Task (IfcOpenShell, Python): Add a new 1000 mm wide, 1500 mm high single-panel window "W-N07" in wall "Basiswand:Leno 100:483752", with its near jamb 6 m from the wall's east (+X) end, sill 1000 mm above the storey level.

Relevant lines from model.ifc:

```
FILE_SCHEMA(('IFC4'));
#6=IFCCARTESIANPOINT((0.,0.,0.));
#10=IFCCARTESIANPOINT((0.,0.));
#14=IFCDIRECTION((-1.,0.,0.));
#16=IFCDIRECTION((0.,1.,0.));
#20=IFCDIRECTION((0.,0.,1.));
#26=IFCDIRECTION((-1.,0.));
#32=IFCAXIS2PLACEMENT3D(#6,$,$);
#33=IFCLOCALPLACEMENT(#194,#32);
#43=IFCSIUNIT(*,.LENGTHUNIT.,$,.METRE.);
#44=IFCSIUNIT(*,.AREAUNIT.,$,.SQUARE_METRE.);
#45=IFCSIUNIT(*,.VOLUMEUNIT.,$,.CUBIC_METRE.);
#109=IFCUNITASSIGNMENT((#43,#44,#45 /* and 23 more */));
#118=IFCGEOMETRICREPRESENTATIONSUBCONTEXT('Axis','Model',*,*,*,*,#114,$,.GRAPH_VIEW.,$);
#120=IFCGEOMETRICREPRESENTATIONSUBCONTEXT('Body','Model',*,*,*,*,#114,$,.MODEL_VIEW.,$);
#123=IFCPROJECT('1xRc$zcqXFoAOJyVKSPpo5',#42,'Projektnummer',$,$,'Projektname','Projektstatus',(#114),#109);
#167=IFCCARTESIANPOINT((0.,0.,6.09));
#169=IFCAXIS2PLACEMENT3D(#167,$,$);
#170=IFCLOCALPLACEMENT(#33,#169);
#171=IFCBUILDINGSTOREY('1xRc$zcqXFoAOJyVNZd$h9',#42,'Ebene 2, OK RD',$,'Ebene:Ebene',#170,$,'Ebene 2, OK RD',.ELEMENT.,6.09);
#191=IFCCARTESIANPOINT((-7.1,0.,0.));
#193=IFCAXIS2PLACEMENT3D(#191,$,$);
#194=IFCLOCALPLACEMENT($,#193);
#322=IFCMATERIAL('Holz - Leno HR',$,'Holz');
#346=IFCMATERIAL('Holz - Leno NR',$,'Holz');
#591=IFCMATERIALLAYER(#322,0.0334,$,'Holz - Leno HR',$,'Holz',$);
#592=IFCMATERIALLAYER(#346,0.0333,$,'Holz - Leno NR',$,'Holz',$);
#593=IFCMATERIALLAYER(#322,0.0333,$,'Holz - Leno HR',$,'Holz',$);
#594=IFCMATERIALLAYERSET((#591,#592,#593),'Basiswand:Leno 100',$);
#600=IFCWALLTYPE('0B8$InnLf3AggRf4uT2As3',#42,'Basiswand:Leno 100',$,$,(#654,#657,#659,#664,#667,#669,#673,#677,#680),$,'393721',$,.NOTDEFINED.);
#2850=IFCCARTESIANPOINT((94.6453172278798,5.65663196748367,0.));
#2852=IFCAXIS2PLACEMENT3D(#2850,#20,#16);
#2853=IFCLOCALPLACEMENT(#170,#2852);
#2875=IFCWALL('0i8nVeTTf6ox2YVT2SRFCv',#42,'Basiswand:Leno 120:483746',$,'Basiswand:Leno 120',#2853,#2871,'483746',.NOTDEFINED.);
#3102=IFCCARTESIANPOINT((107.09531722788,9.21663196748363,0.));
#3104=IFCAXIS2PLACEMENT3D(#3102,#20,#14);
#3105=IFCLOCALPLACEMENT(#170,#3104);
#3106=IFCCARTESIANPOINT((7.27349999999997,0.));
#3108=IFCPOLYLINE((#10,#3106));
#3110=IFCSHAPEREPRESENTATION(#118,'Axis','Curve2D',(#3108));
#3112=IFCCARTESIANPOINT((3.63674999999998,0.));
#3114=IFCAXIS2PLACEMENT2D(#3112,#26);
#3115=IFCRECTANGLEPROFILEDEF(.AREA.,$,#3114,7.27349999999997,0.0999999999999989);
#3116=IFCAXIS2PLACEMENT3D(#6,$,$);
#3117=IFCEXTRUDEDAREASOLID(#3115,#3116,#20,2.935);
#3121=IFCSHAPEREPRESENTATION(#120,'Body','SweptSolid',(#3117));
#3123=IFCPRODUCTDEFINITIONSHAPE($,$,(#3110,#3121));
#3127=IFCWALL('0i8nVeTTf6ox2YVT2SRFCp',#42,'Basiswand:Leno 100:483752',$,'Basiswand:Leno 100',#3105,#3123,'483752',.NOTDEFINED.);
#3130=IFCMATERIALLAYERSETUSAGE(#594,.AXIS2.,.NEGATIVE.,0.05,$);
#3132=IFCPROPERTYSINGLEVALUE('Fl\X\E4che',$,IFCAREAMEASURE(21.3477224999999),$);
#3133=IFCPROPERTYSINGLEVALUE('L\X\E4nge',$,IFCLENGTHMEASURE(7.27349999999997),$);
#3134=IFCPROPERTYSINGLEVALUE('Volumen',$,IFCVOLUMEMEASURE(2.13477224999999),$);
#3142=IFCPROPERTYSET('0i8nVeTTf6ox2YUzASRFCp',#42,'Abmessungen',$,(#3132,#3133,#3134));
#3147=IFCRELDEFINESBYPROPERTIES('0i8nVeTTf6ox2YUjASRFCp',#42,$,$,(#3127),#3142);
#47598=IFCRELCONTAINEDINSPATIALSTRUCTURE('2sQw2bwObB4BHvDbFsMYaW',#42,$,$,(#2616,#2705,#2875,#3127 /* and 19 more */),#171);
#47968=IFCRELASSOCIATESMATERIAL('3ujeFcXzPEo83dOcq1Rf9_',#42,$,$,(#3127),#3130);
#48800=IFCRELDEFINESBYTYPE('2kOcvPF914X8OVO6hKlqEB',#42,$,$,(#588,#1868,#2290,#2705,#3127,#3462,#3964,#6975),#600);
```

```python
import numpy as np
import ifcopenshell
import ifcopenshell.api.feature
import ifcopenshell.api.geometry
import ifcopenshell.api.pset
import ifcopenshell.api.root
import ifcopenshell.api.spatial
import ifcopenshell.geom
import ifcopenshell.util.element
import ifcopenshell.util.placement
import ifcopenshell.util.representation
import ifcopenshell.util.shape
import ifcopenshell.util.unit

model = ifcopenshell.open("model.ifc")
unit_scale = ifcopenshell.util.unit.calculate_unit_scale(model)
area_scale = ifcopenshell.util.unit.calculate_unit_scale(model, "AREAUNIT")
volume_scale = ifcopenshell.util.unit.calculate_unit_scale(model, "VOLUMEUNIT")
settings = ifcopenshell.geom.settings()


def volume(element):
    """Net volume in cubic metres, openings subtracted."""
    shape = ifcopenshell.geom.create_shape(settings, element)
    return ifcopenshell.util.shape.get_volume(shape.geometry)


wall = model.by_guid("0i8nVeTTf6ox2YVT2SRFCp")
storey = ifcopenshell.util.element.get_container(wall, ifc_class="IfcBuildingStorey")
context = ifcopenshell.util.representation.get_context(model, "Model", "Body", "MODEL_VIEW")
before = volume(wall)

width, height, from_end, sill = 1, 1.5, 6, 1  # metres

# The wall runs along its own X axis, and the end named is its -X end.
wall_shape = ifcopenshell.geom.create_shape(settings, wall)
x, y, z = ifcopenshell.util.shape.get_vertices(wall_shape.geometry).T
start = x.min() + from_end
face, thickness = float(y.min()), float(y.max() - y.min())
wall_matrix = ifcopenshell.util.placement.get_local_placement(wall.ObjectPlacement)
level = ifcopenshell.util.placement.get_local_placement(storey.ObjectPlacement)[2, 3]


def in_wall(x, y):
    """Placement at x, y metres in the wall's axes, at sill height."""
    matrix = wall_matrix.copy()
    matrix[:, 3] = wall_matrix @ np.array([x / unit_scale, y / unit_scale, 0.0, 1.0])
    matrix[2, 3] = level + sill / unit_scale
    return matrix


# Opening: a box that overshoots both wall faces by 50 mm.
opening = ifcopenshell.api.root.create_entity(model, ifc_class="IfcOpeningElement", predefined_type="OPENING")
box = ifcopenshell.api.geometry.add_wall_representation(
    model, context=context, length=width, height=height, thickness=thickness + 0.1
)
ifcopenshell.api.geometry.assign_representation(model, product=opening, representation=box)
ifcopenshell.api.geometry.edit_object_placement(model, product=opening, matrix=in_wall(start, face - 0.05), is_si=False)
ifcopenshell.api.feature.add_feature(model, feature=opening, element=wall)

window = ifcopenshell.api.root.create_entity(model, ifc_class="IfcWindow", name="W-N07", predefined_type="WINDOW")
window.OverallWidth, window.OverallHeight = width / unit_scale, height / unit_scale
window.PartitioningType = "SINGLE_PANEL"
body = ifcopenshell.api.geometry.add_window_representation(
    model,
    context=context,
    overall_width=window.OverallWidth,
    overall_height=window.OverallHeight,
    partition_type="SINGLE_PANEL",
)
ifcopenshell.api.geometry.assign_representation(model, product=window, representation=body)
ifcopenshell.api.spatial.assign_container(model, products=[window], relating_structure=storey)
ifcopenshell.api.feature.add_filling(model, opening=opening, element=window)

# Centre the window in the wall's thickness.
ifcopenshell.api.geometry.edit_object_placement(model, product=window, matrix=in_wall(start, face), is_si=False)
window_shape = ifcopenshell.geom.create_shape(settings, window)
depth = ifcopenshell.util.shape.get_vertices(window_shape.geometry)[:, 1]
offset = face + thickness / 2 - (depth.min() + depth.max()) / 2
ifcopenshell.api.geometry.edit_object_placement(model, product=window, matrix=in_wall(start, offset), is_si=False)

after = volume(wall)

# Update the wall's stored quantities.
pset = model.by_id(ifcopenshell.util.element.get_pset(wall, "Abmessungen", should_inherit=False)["id"])
ifcopenshell.api.pset.edit_pset(model, pset=pset, properties={
    "Fläche": model.create_entity("IfcAreaMeasure", after / thickness / area_scale),
    "Volumen": model.create_entity("IfcVolumeMeasure", after / volume_scale),
})

print(f"wall volume {before:.3f} -> {after:.3f} m3")

model.write("model-out.ifc")
```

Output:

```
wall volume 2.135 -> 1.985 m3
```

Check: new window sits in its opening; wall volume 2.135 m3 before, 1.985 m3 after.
